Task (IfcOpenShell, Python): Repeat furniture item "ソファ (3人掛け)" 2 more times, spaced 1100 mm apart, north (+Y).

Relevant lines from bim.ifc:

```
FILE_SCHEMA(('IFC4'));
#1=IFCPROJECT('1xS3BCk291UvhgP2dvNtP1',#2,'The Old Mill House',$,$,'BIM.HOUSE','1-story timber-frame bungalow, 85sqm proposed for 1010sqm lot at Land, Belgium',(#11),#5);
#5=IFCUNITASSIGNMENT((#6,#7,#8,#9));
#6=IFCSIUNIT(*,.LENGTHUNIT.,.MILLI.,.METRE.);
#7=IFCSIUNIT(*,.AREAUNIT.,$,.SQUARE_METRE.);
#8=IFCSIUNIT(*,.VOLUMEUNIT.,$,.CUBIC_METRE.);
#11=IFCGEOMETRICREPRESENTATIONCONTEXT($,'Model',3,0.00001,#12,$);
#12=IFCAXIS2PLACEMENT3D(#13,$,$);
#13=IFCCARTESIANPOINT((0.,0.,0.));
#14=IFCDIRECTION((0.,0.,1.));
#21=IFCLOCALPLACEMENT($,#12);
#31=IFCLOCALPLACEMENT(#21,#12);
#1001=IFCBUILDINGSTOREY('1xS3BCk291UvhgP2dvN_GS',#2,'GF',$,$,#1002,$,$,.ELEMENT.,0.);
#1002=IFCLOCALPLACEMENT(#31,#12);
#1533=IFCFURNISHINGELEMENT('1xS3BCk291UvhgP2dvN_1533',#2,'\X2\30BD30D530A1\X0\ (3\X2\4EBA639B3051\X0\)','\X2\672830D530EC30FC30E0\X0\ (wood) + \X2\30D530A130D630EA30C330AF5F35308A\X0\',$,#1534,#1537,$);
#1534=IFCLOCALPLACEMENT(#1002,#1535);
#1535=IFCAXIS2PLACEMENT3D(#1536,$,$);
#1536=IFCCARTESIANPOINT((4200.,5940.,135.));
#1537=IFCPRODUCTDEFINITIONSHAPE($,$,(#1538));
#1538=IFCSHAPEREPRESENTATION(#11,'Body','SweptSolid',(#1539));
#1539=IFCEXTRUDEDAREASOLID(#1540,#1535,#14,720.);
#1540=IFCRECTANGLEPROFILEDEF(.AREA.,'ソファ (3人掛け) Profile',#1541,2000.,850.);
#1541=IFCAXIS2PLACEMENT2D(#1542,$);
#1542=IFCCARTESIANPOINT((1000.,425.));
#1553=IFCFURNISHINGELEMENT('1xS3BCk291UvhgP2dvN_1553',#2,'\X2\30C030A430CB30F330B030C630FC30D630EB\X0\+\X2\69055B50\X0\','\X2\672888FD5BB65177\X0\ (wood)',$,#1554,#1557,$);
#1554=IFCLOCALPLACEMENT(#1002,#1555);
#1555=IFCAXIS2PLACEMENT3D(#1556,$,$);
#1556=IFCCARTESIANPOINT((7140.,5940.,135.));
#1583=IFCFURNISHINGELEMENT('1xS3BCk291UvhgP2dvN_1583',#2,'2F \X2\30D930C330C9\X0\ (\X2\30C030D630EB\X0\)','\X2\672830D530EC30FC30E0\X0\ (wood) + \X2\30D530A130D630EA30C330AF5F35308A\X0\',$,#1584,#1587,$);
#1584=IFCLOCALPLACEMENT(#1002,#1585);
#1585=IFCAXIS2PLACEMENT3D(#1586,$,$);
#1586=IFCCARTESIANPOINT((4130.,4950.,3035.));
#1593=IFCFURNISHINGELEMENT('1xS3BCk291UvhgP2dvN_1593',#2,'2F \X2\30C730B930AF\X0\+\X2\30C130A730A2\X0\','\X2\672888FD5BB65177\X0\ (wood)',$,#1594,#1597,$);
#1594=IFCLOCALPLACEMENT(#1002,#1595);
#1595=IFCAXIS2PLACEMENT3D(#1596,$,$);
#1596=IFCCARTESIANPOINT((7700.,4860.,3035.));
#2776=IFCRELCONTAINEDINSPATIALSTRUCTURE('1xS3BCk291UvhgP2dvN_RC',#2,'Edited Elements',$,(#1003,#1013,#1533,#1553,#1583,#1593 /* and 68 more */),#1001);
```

```python
import numpy as np
import ifcopenshell
import ifcopenshell.api.geometry
import ifcopenshell.api.root
import ifcopenshell.util.element
import ifcopenshell.util.placement
import ifcopenshell.util.unit

model = ifcopenshell.open("bim.ifc")
unit_scale = ifcopenshell.util.unit.calculate_unit_scale(model)


def reuse_history(source, copy):
    """copy_class also copies each property set's owner history, people and application; keep the originals."""
    for rel in copy.IsDefinedBy:
        if rel.is_a("IfcRelDefinesByProperties") and (history := rel.RelatingPropertyDefinition.OwnerHistory):
            rel.RelatingPropertyDefinition.OwnerHistory = source.OwnerHistory
            ifcopenshell.util.element.remove_deep2(model, history)


source = model.by_id(1533)
base = ifcopenshell.util.placement.get_local_placement(source.ObjectPlacement)
step = np.array([0.0, 1.0, 0.0]) * 1.1 / unit_scale

for i in range(1, 3):
    copy = ifcopenshell.api.root.copy_class(model, product=source)
    copy.Representation = ifcopenshell.util.element.copy_deep(
        model, source.Representation, exclude=["IfcGeometricRepresentationContext", "IfcRepresentationMap"]
    )
    reuse_history(source, copy)
    matrix = base.copy()
    matrix[:3, 3] += i * step
    print("added at", matrix[:3, 3].round(3) + 0.0)
    ifcopenshell.api.geometry.edit_object_placement(model, product=copy, matrix=matrix, is_si=False)

model.write("bim-out.ifc")
```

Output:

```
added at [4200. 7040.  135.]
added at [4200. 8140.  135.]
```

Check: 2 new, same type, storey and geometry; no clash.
